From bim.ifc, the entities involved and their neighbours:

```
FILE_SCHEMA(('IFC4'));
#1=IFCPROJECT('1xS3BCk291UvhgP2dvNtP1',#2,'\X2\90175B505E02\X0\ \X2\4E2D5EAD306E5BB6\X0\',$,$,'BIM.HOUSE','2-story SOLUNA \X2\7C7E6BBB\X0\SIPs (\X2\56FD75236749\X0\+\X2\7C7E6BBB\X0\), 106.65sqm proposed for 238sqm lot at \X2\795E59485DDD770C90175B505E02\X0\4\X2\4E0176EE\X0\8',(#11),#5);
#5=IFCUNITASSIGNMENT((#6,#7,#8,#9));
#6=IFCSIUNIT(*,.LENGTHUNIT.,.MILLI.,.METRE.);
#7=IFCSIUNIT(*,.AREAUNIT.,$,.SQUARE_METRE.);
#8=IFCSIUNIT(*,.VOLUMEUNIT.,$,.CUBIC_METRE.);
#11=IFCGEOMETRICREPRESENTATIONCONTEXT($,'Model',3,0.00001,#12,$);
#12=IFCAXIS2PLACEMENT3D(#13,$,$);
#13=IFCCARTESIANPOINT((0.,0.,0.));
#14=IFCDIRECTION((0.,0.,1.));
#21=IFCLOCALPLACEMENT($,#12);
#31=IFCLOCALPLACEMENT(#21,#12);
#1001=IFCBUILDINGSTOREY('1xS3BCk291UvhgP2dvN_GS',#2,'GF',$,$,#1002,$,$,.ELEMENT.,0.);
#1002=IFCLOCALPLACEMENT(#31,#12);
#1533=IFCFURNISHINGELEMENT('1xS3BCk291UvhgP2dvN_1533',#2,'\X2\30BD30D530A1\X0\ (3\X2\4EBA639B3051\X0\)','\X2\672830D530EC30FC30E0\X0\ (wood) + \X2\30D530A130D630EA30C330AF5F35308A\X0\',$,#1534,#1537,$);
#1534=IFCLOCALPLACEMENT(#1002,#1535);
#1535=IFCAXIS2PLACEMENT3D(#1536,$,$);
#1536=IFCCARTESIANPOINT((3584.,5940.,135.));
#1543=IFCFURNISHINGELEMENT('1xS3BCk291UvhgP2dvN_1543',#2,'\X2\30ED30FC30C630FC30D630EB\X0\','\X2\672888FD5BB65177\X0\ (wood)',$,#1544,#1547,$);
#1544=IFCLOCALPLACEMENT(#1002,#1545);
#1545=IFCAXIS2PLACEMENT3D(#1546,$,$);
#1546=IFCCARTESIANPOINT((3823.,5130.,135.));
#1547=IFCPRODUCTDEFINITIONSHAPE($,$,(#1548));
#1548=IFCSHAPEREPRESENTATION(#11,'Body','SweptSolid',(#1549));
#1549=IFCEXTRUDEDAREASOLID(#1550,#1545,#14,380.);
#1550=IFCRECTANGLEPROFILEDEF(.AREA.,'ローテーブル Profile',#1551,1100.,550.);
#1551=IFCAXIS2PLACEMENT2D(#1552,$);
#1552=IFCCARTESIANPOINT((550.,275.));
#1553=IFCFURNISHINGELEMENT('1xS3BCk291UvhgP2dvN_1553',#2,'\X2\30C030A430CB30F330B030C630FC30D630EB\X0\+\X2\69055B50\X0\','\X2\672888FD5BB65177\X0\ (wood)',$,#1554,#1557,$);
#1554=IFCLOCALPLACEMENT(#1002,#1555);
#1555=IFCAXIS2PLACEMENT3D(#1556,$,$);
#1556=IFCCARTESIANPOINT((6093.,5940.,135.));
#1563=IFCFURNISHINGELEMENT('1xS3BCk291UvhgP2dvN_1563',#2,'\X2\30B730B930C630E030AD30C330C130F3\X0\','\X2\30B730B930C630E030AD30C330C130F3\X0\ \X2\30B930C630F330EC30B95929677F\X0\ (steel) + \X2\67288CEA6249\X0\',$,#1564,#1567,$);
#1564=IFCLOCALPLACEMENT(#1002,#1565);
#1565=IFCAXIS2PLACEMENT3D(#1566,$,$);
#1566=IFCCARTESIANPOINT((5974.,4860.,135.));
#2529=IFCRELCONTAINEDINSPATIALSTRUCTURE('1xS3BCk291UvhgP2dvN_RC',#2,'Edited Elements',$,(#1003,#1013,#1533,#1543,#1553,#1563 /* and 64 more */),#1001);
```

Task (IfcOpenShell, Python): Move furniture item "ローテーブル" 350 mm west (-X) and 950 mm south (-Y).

```python
import ifcopenshell
import ifcopenshell.api.geometry
import ifcopenshell.util.placement

model = ifcopenshell.open("bim.ifc")

item = model.by_guid("1xS3BCk291UvhgP2dvN_1543")
matrix = ifcopenshell.util.placement.get_local_placement(item.ObjectPlacement)
matrix[0, 3] -= 350.0
matrix[1, 3] -= 950.0
ifcopenshell.api.geometry.edit_object_placement(model, product=item, matrix=matrix, is_si=False)

print(ifcopenshell.util.placement.get_local_placement(item.ObjectPlacement).round(3) + 0.0)

model.write("bim_v2.ifc")
```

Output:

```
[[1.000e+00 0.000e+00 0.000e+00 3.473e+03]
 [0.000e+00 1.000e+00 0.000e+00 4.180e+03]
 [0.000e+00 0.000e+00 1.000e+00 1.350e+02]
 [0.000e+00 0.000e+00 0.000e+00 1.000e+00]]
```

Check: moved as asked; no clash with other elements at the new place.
